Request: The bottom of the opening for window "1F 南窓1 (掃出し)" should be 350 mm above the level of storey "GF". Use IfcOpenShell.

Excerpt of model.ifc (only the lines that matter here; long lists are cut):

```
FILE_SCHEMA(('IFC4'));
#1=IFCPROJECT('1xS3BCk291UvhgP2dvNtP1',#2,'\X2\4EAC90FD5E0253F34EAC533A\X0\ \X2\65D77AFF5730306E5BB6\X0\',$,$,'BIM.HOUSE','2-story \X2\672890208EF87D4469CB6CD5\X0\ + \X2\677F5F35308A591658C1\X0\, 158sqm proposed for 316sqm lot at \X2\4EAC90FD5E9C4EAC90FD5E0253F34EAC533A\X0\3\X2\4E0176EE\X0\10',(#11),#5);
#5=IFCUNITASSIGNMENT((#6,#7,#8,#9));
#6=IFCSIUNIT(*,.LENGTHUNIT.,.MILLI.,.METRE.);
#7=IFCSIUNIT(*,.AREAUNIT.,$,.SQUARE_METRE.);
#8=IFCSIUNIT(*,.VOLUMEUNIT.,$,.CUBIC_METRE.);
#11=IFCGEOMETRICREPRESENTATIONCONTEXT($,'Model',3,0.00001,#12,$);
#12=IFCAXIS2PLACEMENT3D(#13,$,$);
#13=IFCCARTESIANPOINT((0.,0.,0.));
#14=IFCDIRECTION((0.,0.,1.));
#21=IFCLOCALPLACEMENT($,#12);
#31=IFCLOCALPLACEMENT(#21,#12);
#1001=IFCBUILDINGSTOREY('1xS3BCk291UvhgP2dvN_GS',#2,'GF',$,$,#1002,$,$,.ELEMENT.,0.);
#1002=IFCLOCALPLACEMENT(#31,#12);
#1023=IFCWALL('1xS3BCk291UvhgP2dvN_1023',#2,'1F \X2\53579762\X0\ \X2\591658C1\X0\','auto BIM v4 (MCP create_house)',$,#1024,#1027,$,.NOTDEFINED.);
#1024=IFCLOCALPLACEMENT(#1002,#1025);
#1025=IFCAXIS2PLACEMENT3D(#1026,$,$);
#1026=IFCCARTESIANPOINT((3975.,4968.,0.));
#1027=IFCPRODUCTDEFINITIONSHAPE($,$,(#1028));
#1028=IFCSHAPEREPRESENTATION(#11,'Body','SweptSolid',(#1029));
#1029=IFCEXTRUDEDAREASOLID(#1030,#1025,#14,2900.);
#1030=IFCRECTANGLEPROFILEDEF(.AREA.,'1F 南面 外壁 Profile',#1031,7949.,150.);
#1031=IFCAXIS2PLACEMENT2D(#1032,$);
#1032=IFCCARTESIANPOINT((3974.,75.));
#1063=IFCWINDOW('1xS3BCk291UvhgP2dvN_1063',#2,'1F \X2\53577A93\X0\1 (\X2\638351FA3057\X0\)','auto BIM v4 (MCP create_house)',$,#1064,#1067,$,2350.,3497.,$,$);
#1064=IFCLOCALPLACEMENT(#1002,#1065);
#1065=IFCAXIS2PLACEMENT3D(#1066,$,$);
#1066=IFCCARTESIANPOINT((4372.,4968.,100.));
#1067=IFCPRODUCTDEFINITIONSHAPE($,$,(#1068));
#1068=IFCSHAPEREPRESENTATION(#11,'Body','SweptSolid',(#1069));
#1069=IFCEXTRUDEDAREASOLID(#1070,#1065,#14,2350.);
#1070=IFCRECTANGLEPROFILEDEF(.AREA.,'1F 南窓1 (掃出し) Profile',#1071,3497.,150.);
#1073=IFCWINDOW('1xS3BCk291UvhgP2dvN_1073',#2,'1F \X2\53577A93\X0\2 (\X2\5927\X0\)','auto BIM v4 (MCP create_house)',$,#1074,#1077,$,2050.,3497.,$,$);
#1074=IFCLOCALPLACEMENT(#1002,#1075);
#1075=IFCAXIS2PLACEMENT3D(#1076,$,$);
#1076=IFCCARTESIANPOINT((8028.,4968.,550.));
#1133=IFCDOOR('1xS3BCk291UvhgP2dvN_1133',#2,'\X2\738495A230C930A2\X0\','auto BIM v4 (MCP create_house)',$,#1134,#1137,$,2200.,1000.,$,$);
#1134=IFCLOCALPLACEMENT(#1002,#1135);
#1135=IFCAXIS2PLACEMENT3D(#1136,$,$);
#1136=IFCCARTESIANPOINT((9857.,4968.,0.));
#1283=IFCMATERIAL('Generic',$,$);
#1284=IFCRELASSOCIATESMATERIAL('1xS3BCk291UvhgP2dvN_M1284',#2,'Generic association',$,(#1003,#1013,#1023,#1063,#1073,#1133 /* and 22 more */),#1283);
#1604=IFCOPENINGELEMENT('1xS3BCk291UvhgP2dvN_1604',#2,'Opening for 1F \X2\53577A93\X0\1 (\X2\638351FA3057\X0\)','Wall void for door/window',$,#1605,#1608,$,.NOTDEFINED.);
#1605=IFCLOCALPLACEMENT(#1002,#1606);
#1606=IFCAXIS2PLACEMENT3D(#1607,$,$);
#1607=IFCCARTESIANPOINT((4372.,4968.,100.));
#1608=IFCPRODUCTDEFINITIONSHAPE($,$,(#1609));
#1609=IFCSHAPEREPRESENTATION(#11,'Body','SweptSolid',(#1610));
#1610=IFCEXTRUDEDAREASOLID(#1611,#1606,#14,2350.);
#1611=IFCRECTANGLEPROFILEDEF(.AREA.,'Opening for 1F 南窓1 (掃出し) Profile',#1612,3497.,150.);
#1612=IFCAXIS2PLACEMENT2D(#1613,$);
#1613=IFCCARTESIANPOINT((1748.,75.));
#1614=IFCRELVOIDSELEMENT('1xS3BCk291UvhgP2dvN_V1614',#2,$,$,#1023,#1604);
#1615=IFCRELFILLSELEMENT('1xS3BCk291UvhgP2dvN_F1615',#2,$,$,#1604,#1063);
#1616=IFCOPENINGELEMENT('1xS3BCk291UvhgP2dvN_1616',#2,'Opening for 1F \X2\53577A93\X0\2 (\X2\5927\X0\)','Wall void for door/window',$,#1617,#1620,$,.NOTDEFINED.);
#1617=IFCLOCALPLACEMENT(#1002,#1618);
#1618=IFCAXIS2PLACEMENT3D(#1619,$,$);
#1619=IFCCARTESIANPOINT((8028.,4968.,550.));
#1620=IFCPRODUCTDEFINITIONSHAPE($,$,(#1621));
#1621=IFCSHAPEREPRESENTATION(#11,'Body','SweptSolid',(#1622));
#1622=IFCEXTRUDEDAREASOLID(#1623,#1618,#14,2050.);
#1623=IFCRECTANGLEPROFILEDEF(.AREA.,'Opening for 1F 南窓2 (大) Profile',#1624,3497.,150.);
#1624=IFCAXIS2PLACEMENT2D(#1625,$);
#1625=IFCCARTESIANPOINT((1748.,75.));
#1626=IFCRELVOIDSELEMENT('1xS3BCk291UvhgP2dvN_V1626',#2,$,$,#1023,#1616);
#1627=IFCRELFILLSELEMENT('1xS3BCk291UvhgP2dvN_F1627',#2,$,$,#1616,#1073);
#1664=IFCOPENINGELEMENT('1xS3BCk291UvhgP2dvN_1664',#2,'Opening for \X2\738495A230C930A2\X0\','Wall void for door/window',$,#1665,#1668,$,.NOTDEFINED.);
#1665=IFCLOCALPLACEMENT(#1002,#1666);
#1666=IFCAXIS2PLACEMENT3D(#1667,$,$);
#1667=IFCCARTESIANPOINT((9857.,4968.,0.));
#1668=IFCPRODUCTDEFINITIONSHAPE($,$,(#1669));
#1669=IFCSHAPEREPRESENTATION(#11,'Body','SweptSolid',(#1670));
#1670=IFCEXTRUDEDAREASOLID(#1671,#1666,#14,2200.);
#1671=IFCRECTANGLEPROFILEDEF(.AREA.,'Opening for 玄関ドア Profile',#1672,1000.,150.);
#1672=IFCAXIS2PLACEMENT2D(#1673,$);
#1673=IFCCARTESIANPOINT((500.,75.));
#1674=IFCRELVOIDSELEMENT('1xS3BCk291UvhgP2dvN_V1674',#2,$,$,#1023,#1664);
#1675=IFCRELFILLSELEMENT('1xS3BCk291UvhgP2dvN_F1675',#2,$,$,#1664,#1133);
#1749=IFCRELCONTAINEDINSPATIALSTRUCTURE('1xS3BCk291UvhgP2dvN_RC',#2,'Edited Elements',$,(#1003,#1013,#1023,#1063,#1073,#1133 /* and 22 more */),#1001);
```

```python
import numpy as np
import ifcopenshell
import ifcopenshell.api.geometry
import ifcopenshell.geom
import ifcopenshell.util.element
import ifcopenshell.util.placement
import ifcopenshell.util.shape
import ifcopenshell.util.unit

model = ifcopenshell.open("model.ifc")
unit_scale = ifcopenshell.util.unit.calculate_unit_scale(model)

window = model.by_guid("1xS3BCk291UvhgP2dvN_1063")
opening = window.FillsVoids[0].RelatingOpeningElement
storey = ifcopenshell.util.element.get_container(window, ifc_class="IfcBuildingStorey")
level = ifcopenshell.util.placement.get_local_placement(storey.ObjectPlacement)[2, 3]

# The opening's origin need not be at the sill, so measure its lowest point.
shape = ifcopenshell.geom.create_shape(ifcopenshell.geom.settings(), opening)
bottom = ifcopenshell.util.shape.get_shape_bottom_elevation(shape, shape.geometry) / unit_scale
dz = level + 350.0 - bottom

shift = np.array([0.0, 0.0, dz])
# The window is not placed relative to its opening, so move both.
for product in (opening, window):
    matrix = ifcopenshell.util.placement.get_local_placement(product.ObjectPlacement)
    matrix[:3, 3] += shift
    ifcopenshell.api.geometry.edit_object_placement(model, product=product, matrix=matrix, is_si=False)

print(f"moved by {dz * unit_scale:+.3f} m")

model.write("model_updated.ifc")
```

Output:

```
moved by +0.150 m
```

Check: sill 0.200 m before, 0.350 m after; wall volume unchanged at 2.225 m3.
